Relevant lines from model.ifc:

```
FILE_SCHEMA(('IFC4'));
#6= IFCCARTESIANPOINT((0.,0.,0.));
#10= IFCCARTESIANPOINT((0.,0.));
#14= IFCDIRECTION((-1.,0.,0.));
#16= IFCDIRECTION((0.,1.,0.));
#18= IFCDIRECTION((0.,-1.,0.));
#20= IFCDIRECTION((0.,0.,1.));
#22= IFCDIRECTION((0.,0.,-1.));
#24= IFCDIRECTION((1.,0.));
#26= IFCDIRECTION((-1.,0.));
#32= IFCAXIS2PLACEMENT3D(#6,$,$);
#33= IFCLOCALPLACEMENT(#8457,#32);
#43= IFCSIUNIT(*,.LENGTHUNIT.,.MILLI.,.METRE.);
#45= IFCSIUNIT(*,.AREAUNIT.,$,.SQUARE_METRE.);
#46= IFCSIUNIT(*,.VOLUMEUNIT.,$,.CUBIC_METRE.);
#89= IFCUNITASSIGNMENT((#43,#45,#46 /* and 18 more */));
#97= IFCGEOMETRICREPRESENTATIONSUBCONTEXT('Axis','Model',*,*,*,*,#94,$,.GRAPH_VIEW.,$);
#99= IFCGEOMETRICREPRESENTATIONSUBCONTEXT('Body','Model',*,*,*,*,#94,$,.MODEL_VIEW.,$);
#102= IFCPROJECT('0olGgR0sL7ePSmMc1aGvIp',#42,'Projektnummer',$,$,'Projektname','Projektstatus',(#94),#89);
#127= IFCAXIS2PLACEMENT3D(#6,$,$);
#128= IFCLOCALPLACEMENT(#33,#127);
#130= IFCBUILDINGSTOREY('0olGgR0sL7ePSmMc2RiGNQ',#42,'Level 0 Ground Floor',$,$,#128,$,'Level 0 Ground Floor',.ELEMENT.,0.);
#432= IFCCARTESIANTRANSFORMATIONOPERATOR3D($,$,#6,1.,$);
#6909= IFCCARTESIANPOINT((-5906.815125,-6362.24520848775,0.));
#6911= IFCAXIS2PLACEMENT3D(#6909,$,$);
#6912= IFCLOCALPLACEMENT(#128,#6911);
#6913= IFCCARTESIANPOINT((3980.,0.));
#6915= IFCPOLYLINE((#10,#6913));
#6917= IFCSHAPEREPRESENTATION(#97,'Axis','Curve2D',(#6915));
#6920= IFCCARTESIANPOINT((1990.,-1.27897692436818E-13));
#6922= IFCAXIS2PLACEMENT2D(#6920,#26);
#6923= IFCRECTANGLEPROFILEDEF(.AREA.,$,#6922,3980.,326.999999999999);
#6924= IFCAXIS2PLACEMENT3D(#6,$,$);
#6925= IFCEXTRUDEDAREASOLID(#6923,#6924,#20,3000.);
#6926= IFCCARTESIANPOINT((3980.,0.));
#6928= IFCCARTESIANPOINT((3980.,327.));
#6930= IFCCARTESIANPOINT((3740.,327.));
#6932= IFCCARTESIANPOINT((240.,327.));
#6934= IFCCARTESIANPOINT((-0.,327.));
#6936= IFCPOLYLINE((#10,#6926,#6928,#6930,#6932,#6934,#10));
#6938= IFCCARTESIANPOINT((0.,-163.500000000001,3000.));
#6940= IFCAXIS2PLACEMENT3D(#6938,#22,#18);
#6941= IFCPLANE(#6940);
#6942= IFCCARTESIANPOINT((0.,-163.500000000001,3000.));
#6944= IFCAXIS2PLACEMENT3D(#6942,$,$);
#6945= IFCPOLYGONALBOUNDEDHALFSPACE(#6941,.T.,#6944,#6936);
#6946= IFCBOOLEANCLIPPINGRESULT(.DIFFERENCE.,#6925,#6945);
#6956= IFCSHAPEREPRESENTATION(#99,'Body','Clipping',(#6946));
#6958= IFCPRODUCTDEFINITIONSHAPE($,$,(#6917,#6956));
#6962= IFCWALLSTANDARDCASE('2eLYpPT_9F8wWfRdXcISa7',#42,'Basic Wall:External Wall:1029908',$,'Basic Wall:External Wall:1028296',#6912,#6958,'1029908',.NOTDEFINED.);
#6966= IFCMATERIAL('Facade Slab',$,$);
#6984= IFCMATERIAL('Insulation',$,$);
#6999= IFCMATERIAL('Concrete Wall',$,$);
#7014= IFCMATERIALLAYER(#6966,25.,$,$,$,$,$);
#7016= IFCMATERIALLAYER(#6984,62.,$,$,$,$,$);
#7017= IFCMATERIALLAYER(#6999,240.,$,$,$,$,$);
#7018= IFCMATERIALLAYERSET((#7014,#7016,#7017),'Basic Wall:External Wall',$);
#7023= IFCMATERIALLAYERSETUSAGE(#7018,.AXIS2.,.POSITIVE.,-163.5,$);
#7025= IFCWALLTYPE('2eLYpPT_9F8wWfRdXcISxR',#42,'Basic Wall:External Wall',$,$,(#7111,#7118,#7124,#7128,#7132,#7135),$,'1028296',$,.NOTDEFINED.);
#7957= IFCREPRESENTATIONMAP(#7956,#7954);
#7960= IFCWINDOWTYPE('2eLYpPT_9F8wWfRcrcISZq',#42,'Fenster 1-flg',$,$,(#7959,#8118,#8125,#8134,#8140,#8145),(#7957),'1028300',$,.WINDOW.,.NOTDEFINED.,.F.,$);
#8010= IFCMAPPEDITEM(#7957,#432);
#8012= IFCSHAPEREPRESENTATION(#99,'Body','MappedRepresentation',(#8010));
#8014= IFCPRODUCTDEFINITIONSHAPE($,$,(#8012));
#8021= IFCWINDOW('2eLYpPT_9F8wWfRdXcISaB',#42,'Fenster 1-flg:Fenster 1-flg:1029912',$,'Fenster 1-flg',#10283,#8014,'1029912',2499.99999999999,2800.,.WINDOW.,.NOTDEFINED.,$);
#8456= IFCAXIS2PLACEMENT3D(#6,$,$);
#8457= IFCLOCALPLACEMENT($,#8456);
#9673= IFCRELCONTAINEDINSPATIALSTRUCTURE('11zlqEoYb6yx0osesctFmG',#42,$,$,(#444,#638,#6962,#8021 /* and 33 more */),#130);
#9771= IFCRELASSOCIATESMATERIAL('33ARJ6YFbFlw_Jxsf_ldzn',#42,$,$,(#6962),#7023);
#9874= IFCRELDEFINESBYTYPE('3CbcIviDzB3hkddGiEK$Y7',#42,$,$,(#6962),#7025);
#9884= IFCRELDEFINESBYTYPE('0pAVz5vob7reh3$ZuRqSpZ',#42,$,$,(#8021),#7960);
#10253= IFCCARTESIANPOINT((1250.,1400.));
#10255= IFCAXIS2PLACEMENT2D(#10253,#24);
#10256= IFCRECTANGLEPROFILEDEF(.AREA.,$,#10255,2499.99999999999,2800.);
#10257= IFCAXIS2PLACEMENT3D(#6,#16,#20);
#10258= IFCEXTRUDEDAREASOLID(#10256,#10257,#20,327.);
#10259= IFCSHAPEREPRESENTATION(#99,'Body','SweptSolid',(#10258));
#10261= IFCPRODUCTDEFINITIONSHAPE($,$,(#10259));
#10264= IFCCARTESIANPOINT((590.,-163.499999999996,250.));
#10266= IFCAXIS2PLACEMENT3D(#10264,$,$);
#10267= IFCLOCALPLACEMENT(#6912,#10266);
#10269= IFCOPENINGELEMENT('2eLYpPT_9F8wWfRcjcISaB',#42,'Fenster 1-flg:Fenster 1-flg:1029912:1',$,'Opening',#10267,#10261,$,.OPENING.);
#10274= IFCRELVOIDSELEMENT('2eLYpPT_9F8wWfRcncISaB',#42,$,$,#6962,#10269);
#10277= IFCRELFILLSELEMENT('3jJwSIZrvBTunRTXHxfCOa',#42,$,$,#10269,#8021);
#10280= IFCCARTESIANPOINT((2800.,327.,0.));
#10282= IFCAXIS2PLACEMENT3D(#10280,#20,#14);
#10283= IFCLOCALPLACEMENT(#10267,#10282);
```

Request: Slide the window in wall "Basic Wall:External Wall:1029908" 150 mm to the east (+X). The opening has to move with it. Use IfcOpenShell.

```python
import ifcopenshell
import ifcopenshell.api.geometry
import ifcopenshell.util.placement

model = ifcopenshell.open("model.ifc")

window = model.by_guid("2eLYpPT_9F8wWfRdXcISaB")
opening = window.FillsVoids[0].RelatingOpeningElement
wall = opening.VoidsElements[0].RelatingBuildingElement

wall_matrix = ifcopenshell.util.placement.get_local_placement(wall.ObjectPlacement)
shift = wall_matrix[:3, 0] * 150.0
before = ifcopenshell.util.placement.get_local_placement(window.ObjectPlacement)[:3, 3].copy()

# The window is placed relative to its opening, so it follows when the opening moves.
matrix = ifcopenshell.util.placement.get_local_placement(opening.ObjectPlacement)
matrix[:3, 3] += shift
ifcopenshell.api.geometry.edit_object_placement(
    model, product=opening, matrix=matrix, is_si=False, should_transform_children=True
)

after = ifcopenshell.util.placement.get_local_placement(window.ObjectPlacement)[:3, 3]
print("window moved by", (after - before).round(3) + 0.0)

model.write("model-out.ifc")
```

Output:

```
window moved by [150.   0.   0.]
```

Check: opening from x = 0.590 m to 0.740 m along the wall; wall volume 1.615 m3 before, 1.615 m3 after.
